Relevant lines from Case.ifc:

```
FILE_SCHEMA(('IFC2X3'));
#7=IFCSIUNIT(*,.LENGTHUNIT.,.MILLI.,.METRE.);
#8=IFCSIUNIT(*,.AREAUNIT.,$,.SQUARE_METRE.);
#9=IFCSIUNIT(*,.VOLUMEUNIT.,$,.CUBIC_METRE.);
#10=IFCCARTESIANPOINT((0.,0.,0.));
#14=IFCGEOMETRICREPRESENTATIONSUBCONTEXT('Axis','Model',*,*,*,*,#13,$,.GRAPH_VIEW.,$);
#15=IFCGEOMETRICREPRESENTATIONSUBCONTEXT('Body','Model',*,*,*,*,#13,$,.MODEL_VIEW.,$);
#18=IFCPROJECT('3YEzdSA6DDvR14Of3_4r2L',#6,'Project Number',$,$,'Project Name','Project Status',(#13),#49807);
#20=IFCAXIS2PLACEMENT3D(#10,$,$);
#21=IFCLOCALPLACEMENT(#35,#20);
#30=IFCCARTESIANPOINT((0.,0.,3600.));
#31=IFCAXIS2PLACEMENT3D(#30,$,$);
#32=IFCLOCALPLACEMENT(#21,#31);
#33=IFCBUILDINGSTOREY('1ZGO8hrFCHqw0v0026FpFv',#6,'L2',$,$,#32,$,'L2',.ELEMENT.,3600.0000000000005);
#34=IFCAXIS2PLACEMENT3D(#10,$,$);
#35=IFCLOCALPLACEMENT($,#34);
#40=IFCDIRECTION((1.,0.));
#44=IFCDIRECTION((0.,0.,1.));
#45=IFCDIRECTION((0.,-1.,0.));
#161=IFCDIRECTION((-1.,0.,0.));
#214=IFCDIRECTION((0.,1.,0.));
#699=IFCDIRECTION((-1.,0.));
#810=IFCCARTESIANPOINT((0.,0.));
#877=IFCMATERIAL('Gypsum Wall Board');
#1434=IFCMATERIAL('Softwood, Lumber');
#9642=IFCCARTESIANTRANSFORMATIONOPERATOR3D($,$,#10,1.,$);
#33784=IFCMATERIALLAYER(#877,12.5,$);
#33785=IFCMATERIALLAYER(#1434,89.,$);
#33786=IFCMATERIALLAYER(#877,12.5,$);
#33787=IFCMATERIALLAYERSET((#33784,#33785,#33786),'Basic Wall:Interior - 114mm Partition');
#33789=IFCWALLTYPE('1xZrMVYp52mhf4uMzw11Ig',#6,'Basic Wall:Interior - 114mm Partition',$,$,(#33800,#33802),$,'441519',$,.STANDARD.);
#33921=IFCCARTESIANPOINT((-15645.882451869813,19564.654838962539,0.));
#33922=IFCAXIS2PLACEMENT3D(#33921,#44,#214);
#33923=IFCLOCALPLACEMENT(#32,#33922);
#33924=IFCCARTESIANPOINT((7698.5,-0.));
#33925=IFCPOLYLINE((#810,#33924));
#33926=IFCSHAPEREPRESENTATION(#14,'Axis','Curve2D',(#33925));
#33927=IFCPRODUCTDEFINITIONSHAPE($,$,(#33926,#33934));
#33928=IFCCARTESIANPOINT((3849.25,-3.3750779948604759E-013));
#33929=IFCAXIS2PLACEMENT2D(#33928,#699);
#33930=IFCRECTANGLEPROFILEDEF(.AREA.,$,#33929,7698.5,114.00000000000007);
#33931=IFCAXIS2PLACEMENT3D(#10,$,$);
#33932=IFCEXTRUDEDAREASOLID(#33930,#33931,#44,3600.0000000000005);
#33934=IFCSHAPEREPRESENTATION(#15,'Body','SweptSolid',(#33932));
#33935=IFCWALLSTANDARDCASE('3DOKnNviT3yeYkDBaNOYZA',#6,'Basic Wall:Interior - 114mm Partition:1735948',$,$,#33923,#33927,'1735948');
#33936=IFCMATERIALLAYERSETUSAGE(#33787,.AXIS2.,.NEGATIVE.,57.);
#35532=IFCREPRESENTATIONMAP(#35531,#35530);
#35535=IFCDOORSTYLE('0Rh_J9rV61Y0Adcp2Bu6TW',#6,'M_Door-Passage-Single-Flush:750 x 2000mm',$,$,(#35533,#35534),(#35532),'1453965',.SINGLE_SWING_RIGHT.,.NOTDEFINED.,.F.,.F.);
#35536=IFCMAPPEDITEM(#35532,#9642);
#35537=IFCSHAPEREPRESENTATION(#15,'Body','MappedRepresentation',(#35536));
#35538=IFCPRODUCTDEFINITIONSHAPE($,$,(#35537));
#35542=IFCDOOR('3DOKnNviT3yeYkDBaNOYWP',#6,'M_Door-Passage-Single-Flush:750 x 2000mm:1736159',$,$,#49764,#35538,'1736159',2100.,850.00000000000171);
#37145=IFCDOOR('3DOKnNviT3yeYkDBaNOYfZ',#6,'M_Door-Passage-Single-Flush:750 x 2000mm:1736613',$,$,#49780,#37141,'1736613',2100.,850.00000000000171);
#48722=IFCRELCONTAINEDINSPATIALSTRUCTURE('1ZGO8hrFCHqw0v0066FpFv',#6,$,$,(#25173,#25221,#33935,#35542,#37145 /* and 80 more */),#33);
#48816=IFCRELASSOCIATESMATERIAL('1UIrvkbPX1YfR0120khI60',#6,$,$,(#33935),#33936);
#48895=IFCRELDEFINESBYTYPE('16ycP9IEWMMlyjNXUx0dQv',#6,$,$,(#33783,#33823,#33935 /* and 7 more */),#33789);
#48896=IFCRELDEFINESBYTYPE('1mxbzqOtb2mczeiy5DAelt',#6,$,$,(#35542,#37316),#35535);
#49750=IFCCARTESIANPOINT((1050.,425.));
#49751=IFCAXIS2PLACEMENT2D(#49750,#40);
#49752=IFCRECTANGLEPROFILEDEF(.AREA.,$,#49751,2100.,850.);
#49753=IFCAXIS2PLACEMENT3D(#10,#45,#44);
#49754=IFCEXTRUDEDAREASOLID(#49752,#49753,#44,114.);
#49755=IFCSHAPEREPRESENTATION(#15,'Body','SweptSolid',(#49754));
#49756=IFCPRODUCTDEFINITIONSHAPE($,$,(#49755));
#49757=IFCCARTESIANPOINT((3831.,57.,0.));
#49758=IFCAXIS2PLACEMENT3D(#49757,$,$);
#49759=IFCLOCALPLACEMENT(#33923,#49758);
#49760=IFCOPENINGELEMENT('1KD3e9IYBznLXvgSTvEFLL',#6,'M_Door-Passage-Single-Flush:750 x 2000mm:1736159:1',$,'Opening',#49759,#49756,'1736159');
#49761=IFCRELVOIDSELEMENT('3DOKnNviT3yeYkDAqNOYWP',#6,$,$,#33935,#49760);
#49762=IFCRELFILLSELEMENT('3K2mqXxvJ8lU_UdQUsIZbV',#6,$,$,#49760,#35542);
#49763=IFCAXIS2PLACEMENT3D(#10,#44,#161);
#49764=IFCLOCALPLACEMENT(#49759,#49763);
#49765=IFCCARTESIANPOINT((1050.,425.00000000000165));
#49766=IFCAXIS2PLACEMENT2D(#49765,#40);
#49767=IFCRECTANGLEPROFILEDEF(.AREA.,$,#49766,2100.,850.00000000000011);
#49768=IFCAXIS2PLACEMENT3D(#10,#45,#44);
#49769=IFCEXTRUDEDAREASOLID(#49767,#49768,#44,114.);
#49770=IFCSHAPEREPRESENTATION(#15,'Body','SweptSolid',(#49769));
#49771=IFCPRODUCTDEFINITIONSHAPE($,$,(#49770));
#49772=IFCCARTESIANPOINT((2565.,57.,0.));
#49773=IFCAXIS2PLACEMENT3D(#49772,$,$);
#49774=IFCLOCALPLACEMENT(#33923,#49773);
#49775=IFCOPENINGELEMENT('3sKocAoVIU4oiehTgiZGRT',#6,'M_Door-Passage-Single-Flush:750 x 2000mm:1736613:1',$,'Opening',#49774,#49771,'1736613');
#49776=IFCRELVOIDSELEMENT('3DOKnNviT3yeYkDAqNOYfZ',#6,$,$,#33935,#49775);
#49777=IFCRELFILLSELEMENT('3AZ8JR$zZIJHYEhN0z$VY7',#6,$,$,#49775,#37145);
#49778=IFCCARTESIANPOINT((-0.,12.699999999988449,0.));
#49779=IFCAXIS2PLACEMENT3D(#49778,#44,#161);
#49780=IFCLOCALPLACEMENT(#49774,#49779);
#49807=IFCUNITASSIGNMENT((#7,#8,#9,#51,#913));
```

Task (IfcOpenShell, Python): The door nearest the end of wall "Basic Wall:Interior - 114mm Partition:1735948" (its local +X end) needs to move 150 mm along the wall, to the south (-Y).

```python
import ifcopenshell
import ifcopenshell.api.geometry
import ifcopenshell.util.placement
import ifcopenshell.util.unit

model = ifcopenshell.open("Case.ifc")
unit_scale = ifcopenshell.util.unit.calculate_unit_scale(model)

door = model.by_id(35542)
opening = door.FillsVoids[0].RelatingOpeningElement
wall = opening.VoidsElements[0].RelatingBuildingElement

wall_matrix = ifcopenshell.util.placement.get_local_placement(wall.ObjectPlacement)
shift = wall_matrix[:3, 0] * -0.15 / unit_scale
before = ifcopenshell.util.placement.get_local_placement(door.ObjectPlacement)[:3, 3].copy()

# The door is placed relative to its opening, so it follows when the opening moves.
matrix = ifcopenshell.util.placement.get_local_placement(opening.ObjectPlacement)
matrix[:3, 3] += shift
ifcopenshell.api.geometry.edit_object_placement(
    model, product=opening, matrix=matrix, is_si=False, should_transform_children=True
)

after = ifcopenshell.util.placement.get_local_placement(door.ObjectPlacement)[:3, 3]
print("door moved by", (after - before).round(3) + 0.0)

model.write("Case-out.ifc")
```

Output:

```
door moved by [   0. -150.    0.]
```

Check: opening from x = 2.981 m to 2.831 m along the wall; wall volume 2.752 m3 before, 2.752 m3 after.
